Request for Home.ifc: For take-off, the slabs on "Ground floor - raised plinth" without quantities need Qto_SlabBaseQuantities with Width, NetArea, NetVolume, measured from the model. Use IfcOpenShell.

First a look at what the model holds.

```python
import ifcopenshell
import ifcopenshell.util.element
import ifcopenshell.util.unit

model = ifcopenshell.open("Home.ifc")
print(model.schema)
for unit_type in ("LENGTHUNIT", "AREAUNIT", "VOLUMEUNIT"):
    print(unit_type, ifcopenshell.util.unit.calculate_unit_scale(model, unit_type))
storey = next(s for s in model.by_type("IfcBuildingStorey") if s.Name == "Ground floor - raised plinth")
slabs = [e for e in ifcopenshell.util.element.get_decomposition(storey) if e.is_a("IfcSlab")]
for e in sorted(slabs, key=lambda e: e.id()):
    print(e.id(), e.is_a(), e.Name, list(ifcopenshell.util.element.get_psets(e, qtos_only=True)), sep=" | ")
```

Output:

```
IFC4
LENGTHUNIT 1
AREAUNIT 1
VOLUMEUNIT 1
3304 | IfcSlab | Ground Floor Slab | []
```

```python
import ifcopenshell
import ifcopenshell.api.pset
import ifcopenshell.geom
import ifcopenshell.util.element
import ifcopenshell.util.shape
import ifcopenshell.util.unit

model = ifcopenshell.open("Home.ifc")
unit_scale = ifcopenshell.util.unit.calculate_unit_scale(model)
area_scale = ifcopenshell.util.unit.calculate_unit_scale(model, "AREAUNIT")
volume_scale = ifcopenshell.util.unit.calculate_unit_scale(model, "VOLUMEUNIT")
settings = ifcopenshell.geom.settings()

storey = next(s for s in model.by_type("IfcBuildingStorey") if s.Name == "Ground floor - raised plinth")
slabs = [e for e in ifcopenshell.util.element.get_decomposition(storey) if e.is_a("IfcSlab")]

for e in sorted(slabs, key=lambda e: e.id()):
    if ifcopenshell.util.element.get_psets(e, qtos_only=True, should_inherit=False):
        continue
    # Geometry comes back in metres, in the element's own axes.
    shape = ifcopenshell.geom.create_shape(settings, e)
    values = {
        "Width": ifcopenshell.util.shape.get_z(shape.geometry) / unit_scale,
        "NetArea": ifcopenshell.util.shape.get_footprint_area(shape.geometry) / area_scale,
        "NetVolume": ifcopenshell.util.shape.get_volume(shape.geometry) / volume_scale,
    }
    qto = ifcopenshell.api.pset.add_qto(model, product=e, name="Qto_SlabBaseQuantities")
    ifcopenshell.api.pset.edit_qto(model, qto=qto, properties=values)
    print(e.id(), {k: round(v, 3) for k, v in values.items()})

model.write("Home_edited.ifc")
```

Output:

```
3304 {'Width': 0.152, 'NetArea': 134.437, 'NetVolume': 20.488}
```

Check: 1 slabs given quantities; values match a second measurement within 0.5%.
